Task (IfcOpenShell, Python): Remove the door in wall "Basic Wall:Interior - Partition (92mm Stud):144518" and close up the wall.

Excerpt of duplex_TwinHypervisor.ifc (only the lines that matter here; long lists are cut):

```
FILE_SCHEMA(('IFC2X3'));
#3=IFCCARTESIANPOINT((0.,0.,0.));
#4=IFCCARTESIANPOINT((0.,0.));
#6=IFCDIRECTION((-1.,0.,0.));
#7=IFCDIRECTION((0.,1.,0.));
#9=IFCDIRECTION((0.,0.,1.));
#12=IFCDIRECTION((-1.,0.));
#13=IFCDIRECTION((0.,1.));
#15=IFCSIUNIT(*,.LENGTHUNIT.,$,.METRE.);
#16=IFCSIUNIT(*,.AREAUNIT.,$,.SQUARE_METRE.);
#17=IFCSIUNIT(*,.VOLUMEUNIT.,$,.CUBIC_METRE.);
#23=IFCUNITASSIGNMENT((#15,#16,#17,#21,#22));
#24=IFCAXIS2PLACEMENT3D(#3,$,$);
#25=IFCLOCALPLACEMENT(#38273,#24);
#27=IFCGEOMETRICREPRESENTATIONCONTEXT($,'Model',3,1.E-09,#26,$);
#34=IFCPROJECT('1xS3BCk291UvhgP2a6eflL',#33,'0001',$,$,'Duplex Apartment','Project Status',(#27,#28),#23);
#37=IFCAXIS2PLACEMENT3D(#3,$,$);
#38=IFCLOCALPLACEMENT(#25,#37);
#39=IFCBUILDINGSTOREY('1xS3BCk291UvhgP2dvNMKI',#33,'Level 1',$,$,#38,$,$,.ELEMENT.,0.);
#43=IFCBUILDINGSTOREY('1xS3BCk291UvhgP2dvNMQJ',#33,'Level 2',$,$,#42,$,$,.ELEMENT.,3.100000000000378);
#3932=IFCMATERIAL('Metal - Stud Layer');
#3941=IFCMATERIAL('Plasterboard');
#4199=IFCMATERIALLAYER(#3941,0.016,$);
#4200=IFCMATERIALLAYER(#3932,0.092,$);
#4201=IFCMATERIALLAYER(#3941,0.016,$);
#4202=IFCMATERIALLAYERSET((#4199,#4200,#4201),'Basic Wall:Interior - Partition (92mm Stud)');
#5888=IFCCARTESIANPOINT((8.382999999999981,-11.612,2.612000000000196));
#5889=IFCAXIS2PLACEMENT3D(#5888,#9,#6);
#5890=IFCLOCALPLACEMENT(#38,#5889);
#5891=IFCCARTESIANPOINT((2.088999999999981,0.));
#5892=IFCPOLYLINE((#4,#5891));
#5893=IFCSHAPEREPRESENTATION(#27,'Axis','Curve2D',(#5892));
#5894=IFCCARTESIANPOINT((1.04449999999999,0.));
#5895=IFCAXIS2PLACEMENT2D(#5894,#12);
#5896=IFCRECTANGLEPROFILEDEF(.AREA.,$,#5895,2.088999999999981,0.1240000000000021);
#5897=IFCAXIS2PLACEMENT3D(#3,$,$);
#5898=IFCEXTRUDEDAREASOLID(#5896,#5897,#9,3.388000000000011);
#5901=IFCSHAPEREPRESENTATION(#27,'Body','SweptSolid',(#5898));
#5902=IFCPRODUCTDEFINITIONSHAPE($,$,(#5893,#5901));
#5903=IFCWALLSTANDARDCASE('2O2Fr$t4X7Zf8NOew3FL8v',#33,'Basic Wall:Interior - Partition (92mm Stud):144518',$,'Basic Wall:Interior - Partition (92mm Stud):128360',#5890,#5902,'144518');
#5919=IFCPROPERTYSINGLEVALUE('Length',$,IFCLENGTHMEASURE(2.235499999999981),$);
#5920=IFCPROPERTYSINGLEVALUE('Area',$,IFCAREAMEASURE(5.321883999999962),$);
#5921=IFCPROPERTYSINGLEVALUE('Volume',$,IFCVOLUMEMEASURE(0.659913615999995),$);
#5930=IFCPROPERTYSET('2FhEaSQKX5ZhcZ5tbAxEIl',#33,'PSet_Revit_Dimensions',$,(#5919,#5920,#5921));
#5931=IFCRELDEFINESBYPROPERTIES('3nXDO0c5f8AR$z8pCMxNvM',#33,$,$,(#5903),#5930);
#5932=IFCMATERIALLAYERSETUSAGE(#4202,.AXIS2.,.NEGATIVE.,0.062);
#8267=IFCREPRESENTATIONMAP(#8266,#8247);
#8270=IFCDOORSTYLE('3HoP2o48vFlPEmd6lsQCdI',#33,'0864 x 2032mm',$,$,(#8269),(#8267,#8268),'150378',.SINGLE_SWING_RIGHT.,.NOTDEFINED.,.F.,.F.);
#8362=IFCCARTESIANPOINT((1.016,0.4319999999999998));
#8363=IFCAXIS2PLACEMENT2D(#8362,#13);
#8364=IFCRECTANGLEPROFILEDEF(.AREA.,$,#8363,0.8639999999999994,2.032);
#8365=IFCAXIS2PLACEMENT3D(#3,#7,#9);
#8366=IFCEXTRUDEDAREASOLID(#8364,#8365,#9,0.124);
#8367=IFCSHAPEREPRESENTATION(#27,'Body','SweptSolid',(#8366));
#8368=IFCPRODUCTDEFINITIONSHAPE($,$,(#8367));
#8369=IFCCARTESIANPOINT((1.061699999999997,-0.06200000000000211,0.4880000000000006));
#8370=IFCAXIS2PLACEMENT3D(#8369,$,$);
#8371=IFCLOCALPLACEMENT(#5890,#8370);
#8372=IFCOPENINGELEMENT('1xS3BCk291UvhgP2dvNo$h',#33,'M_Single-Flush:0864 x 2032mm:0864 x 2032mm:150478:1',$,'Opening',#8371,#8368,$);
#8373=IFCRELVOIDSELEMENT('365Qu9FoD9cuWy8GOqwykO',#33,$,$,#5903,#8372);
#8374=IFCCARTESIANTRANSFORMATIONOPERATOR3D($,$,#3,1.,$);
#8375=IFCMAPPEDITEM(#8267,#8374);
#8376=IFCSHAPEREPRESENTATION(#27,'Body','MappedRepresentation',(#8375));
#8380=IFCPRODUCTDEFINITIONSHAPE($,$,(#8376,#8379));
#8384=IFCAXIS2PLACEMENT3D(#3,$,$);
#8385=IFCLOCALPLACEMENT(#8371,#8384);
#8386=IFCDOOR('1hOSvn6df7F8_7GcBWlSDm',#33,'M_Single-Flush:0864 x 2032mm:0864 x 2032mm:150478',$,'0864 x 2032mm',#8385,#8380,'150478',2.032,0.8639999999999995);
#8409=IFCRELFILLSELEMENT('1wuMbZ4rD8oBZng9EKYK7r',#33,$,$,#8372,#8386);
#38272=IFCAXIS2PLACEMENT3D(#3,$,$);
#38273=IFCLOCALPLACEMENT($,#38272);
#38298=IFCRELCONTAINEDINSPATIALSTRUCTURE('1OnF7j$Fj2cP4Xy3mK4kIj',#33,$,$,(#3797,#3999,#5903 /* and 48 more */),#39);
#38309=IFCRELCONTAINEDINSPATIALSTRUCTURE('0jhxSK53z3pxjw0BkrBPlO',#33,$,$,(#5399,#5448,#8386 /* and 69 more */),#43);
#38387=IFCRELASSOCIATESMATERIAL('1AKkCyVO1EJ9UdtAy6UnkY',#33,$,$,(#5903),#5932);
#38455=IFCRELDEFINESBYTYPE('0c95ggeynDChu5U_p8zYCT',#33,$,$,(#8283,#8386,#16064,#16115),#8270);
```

```python
import ifcopenshell
import ifcopenshell.api.feature
import ifcopenshell.api.pset
import ifcopenshell.api.root
import ifcopenshell.geom
import ifcopenshell.util.element
import ifcopenshell.util.shape
import ifcopenshell.util.unit

model = ifcopenshell.open("duplex_TwinHypervisor.ifc")
area_scale = ifcopenshell.util.unit.calculate_unit_scale(model, "AREAUNIT")
volume_scale = ifcopenshell.util.unit.calculate_unit_scale(model, "VOLUMEUNIT")
settings = ifcopenshell.geom.settings()


def volume(element):
    """Net volume in cubic metres, openings subtracted."""
    shape = ifcopenshell.geom.create_shape(settings, element)
    return ifcopenshell.util.shape.get_volume(shape.geometry)


door = model.by_guid("1hOSvn6df7F8_7GcBWlSDm")
opening = door.FillsVoids[0].RelatingOpeningElement
wall = opening.VoidsElements[0].RelatingBuildingElement
before = volume(wall)

ifcopenshell.api.root.remove_product(model, product=door)
ifcopenshell.api.feature.remove_feature(model, feature=opening)

after = volume(wall)
thickness = 0.124  # wall thickness in metres

# Update the wall's stored quantities.
pset = model.by_id(ifcopenshell.util.element.get_pset(wall, "PSet_Revit_Dimensions", should_inherit=False)["id"])
ifcopenshell.api.pset.edit_pset(model, pset=pset, properties={
    "Area": model.create_entity("IfcAreaMeasure", after / thickness / area_scale),
    "Volume": model.create_entity("IfcVolumeMeasure", after / volume_scale),
})

print(f"wall volume {before:.3f} -> {after:.3f} m3")

model.write("duplex_TwinHypervisor_updated.ifc")
```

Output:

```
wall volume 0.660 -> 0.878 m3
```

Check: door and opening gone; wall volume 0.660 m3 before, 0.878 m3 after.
